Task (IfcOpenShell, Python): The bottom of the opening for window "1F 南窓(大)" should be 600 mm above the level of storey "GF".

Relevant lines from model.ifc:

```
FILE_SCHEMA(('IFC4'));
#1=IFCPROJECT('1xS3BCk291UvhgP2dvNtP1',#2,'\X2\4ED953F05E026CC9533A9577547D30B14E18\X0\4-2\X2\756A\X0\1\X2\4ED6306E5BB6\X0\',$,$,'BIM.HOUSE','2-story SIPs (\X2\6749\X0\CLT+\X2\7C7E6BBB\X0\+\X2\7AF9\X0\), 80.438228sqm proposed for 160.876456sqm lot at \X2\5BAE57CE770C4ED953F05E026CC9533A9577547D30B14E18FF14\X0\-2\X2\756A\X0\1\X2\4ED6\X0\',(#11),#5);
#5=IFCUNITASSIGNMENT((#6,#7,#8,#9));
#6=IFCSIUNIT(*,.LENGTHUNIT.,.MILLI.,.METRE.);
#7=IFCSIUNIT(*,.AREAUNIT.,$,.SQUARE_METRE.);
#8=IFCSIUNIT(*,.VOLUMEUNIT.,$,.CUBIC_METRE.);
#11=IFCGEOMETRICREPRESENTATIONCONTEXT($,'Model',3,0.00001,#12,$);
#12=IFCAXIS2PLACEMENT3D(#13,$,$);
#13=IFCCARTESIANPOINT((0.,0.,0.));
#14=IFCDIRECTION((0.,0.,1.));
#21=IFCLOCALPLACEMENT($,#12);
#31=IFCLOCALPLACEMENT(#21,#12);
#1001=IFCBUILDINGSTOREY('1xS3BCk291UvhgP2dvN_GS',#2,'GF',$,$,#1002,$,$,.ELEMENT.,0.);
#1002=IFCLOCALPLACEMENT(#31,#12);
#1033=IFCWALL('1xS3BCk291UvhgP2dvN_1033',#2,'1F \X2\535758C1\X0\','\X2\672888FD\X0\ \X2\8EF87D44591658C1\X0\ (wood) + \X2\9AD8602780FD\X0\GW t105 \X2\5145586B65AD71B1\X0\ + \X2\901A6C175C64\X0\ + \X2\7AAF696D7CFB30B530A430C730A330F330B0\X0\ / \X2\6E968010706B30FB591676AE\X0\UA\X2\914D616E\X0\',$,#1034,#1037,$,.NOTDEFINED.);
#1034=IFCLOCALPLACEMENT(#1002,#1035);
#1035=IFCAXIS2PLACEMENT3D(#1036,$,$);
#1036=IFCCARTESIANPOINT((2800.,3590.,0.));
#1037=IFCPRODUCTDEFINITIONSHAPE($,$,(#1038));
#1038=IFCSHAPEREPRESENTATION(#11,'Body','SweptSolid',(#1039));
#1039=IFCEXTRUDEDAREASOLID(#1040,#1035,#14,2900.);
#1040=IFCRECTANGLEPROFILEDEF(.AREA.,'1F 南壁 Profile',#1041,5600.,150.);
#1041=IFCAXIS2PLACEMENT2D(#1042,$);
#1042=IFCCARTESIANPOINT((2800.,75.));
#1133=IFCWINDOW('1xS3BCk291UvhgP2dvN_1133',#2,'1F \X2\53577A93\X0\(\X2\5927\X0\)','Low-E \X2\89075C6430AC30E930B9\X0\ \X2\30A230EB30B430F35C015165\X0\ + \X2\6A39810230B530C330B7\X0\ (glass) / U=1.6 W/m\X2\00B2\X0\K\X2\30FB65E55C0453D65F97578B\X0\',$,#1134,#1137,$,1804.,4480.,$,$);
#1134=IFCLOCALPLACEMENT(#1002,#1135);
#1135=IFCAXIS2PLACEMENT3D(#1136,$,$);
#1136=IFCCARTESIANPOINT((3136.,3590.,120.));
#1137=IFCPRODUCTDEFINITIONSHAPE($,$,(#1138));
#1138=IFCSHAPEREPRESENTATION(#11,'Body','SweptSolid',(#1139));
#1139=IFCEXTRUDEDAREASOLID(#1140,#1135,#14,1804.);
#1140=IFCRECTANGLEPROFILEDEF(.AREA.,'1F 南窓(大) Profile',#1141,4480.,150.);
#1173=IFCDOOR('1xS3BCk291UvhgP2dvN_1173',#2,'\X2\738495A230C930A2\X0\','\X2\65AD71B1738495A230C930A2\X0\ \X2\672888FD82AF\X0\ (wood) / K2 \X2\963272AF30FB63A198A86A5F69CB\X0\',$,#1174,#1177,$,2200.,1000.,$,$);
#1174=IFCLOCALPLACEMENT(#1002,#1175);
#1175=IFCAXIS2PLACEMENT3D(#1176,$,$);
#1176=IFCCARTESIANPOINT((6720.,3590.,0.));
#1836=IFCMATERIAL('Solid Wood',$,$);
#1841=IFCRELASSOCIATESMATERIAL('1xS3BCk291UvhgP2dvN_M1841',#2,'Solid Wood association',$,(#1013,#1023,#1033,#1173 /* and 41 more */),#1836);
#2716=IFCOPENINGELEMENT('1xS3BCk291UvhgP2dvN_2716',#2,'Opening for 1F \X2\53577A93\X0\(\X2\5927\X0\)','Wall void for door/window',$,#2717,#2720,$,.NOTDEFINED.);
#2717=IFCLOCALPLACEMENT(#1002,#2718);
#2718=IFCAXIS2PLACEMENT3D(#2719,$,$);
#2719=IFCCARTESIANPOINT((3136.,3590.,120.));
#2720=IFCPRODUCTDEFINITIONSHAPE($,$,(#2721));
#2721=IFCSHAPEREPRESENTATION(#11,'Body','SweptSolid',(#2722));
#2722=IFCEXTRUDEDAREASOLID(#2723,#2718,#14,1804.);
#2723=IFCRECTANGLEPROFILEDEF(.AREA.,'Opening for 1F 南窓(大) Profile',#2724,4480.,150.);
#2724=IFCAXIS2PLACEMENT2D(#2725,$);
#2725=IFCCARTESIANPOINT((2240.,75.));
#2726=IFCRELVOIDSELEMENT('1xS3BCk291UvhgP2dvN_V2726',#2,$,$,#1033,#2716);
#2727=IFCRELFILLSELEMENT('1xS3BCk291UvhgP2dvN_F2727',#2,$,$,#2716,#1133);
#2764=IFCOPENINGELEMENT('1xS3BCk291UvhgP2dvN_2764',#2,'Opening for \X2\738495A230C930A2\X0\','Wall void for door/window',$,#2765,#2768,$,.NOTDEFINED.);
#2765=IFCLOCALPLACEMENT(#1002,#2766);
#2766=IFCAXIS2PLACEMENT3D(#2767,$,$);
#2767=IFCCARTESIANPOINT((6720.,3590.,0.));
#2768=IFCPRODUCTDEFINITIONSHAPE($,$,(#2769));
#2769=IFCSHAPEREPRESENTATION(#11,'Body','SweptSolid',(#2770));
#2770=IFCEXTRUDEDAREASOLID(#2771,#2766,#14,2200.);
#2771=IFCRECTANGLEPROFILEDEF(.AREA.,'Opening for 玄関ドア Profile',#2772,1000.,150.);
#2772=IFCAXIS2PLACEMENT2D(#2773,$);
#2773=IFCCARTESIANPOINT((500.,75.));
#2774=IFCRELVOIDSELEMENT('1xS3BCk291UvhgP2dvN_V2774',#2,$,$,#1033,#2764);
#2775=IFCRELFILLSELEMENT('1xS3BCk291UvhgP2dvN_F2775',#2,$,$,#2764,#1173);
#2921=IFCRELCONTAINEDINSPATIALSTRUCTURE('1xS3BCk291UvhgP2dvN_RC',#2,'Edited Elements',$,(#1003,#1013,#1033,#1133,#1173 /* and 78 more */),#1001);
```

```python
import numpy as np
import ifcopenshell
import ifcopenshell.api.geometry
import ifcopenshell.geom
import ifcopenshell.util.element
import ifcopenshell.util.placement
import ifcopenshell.util.shape
import ifcopenshell.util.unit

model = ifcopenshell.open("model.ifc")
unit_scale = ifcopenshell.util.unit.calculate_unit_scale(model)

window = model.by_guid("1xS3BCk291UvhgP2dvN_1133")
opening = window.FillsVoids[0].RelatingOpeningElement
storey = ifcopenshell.util.element.get_container(window, ifc_class="IfcBuildingStorey")
level = ifcopenshell.util.placement.get_local_placement(storey.ObjectPlacement)[2, 3]

# The opening's origin need not be at the sill, so measure its lowest point.
shape = ifcopenshell.geom.create_shape(ifcopenshell.geom.settings(), opening)
bottom = ifcopenshell.util.shape.get_shape_bottom_elevation(shape, shape.geometry) / unit_scale
dz = level + 600.0 - bottom

shift = np.array([0.0, 0.0, dz])
# The window is not placed relative to its opening, so move both.
for product in (opening, window):
    matrix = ifcopenshell.util.placement.get_local_placement(product.ObjectPlacement)
    matrix[:3, 3] += shift
    ifcopenshell.api.geometry.edit_object_placement(model, product=product, matrix=matrix, is_si=False)

print(f"moved by {dz * unit_scale:+.3f} m")

model.write("model_rev.ifc")
```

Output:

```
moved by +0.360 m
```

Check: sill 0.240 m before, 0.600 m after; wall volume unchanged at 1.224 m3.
